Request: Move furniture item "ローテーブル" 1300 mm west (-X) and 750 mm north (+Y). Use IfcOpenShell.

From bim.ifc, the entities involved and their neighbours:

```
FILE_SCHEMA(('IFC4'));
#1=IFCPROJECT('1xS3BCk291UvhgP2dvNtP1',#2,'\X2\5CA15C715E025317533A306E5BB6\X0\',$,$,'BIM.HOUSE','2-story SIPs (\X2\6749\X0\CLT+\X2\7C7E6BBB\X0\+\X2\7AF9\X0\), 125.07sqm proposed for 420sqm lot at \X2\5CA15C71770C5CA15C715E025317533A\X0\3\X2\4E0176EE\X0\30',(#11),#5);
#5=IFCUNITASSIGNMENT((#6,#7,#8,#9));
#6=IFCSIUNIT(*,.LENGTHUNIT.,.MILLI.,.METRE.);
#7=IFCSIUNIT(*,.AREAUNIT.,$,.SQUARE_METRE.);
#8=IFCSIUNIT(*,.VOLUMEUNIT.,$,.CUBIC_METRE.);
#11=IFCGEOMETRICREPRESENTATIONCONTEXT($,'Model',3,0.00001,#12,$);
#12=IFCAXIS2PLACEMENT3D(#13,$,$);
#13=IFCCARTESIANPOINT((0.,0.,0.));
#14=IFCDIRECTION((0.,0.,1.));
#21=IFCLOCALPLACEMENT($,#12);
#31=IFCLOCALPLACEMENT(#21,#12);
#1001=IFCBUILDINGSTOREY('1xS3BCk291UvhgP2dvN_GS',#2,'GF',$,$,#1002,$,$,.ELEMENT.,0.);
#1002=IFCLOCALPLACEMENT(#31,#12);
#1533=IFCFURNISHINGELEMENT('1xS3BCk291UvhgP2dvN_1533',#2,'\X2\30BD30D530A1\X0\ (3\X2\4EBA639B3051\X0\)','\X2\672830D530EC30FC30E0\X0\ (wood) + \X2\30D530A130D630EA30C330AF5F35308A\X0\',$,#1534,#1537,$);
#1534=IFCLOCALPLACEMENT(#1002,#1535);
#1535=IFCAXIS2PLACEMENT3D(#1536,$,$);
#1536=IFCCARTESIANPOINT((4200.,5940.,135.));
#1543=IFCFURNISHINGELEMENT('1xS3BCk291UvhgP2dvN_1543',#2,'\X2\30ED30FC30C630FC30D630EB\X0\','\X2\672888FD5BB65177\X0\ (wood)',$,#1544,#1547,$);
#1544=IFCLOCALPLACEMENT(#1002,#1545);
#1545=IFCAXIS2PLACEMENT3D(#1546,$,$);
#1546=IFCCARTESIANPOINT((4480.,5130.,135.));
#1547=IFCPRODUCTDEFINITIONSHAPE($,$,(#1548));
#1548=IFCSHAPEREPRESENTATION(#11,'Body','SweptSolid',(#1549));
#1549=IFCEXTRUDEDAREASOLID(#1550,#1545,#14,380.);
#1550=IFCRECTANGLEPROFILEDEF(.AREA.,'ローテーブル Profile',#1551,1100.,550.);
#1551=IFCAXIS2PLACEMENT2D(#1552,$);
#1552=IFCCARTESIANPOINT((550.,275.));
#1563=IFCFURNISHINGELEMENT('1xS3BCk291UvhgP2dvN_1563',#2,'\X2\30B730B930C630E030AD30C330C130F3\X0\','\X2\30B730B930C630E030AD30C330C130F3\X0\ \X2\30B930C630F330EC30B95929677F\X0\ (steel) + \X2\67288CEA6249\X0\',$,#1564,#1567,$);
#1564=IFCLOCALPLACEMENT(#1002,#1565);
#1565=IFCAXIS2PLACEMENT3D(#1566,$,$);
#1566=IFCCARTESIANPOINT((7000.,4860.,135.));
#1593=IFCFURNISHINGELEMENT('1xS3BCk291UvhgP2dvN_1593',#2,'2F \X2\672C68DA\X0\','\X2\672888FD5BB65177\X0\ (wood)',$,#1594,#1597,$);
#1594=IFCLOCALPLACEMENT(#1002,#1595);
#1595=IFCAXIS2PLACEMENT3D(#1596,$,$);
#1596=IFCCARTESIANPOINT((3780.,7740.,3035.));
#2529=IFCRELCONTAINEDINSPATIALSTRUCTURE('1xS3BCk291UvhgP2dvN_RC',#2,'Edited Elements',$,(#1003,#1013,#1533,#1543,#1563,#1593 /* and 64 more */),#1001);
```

```python
import ifcopenshell
import ifcopenshell.api.geometry
import ifcopenshell.util.placement
import ifcopenshell.util.unit

model = ifcopenshell.open("bim.ifc")
unit_scale = ifcopenshell.util.unit.calculate_unit_scale(model)

item = model.by_guid("1xS3BCk291UvhgP2dvN_1543")
matrix = ifcopenshell.util.placement.get_local_placement(item.ObjectPlacement)
matrix[0, 3] -= 1.3 / unit_scale
matrix[1, 3] += 0.75 / unit_scale
ifcopenshell.api.geometry.edit_object_placement(model, product=item, matrix=matrix, is_si=False)

print(ifcopenshell.util.placement.get_local_placement(item.ObjectPlacement).round(3) + 0.0)

model.write("bim-out.ifc")
```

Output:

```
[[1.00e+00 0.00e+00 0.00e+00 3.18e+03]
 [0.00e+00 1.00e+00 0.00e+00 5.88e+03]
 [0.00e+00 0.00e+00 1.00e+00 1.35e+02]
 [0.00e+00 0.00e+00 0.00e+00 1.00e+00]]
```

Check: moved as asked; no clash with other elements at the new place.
